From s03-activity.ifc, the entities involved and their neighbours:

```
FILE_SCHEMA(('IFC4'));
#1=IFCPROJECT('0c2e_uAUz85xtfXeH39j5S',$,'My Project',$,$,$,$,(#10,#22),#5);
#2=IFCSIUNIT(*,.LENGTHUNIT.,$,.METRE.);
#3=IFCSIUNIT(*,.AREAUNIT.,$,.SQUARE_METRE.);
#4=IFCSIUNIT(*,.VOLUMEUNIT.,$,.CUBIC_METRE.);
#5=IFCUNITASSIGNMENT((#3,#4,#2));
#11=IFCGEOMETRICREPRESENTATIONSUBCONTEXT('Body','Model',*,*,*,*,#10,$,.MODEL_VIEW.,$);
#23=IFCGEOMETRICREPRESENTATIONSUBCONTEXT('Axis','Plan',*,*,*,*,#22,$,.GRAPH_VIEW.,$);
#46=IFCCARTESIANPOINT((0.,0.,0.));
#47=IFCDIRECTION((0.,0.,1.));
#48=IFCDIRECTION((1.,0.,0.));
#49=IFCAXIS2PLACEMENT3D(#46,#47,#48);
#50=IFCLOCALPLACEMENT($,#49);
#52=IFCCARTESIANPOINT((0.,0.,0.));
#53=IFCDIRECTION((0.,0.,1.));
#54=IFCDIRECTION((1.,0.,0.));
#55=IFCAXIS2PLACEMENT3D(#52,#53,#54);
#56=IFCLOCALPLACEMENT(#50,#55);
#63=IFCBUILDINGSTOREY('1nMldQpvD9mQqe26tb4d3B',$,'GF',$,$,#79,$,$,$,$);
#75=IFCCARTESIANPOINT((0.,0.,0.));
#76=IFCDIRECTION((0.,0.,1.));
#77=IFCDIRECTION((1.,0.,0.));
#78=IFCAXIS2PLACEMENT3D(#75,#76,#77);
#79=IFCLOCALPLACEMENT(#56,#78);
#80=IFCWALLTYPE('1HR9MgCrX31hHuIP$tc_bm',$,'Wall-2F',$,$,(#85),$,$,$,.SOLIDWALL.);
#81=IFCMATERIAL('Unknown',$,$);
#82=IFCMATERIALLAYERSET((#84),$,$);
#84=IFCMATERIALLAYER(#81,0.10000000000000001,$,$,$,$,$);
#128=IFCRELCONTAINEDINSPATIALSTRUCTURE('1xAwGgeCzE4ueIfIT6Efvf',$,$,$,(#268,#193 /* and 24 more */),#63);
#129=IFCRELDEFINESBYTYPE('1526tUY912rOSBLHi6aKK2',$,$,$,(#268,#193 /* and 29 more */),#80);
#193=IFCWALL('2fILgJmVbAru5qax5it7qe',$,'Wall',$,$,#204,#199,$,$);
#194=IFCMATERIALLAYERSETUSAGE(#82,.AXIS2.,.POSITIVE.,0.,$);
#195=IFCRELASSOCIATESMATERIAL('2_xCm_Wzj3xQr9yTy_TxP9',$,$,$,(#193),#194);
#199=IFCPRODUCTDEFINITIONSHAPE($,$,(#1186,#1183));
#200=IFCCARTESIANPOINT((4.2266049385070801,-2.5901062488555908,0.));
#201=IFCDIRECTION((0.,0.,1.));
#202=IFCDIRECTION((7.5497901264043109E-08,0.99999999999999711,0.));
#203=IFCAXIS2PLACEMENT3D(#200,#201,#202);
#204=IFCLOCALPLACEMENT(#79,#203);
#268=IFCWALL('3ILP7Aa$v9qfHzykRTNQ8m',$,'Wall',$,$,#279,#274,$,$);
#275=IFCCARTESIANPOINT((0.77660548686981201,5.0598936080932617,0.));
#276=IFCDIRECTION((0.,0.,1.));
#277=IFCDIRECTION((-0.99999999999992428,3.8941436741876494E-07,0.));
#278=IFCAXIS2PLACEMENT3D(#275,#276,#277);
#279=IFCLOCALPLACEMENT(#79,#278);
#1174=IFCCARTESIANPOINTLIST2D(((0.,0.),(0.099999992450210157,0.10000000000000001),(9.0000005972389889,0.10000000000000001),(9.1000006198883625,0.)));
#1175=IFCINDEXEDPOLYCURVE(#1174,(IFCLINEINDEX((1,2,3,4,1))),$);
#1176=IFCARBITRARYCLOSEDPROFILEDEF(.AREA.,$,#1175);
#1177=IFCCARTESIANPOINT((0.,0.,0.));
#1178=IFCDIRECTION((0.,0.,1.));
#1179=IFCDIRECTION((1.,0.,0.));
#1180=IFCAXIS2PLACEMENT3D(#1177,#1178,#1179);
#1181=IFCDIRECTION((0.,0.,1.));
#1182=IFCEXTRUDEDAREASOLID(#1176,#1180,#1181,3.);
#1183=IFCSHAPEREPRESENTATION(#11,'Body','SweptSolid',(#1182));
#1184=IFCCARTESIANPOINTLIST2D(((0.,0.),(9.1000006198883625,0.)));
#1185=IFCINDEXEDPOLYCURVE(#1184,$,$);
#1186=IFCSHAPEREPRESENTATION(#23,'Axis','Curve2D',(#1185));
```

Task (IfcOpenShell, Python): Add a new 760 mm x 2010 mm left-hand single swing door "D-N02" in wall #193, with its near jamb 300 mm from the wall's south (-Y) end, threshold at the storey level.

```python
import numpy as np
import ifcopenshell
import ifcopenshell.api.feature
import ifcopenshell.api.geometry
import ifcopenshell.api.root
import ifcopenshell.api.spatial
import ifcopenshell.geom
import ifcopenshell.util.element
import ifcopenshell.util.placement
import ifcopenshell.util.representation
import ifcopenshell.util.shape
import ifcopenshell.util.unit

model = ifcopenshell.open("s03-activity.ifc")
unit_scale = ifcopenshell.util.unit.calculate_unit_scale(model)
settings = ifcopenshell.geom.settings()


def volume(element):
    """Net volume in cubic metres, openings subtracted."""
    shape = ifcopenshell.geom.create_shape(settings, element)
    return ifcopenshell.util.shape.get_volume(shape.geometry)


wall = model.by_guid("2fILgJmVbAru5qax5it7qe")
storey = ifcopenshell.util.element.get_container(wall, ifc_class="IfcBuildingStorey")
context = ifcopenshell.util.representation.get_context(model, "Model", "Body", "MODEL_VIEW")
before = volume(wall)

width, height, from_end, sill = 0.76, 2.01, 0.3, 0.0  # metres

# The wall runs along its own X axis, and the end named is its -X end.
wall_shape = ifcopenshell.geom.create_shape(settings, wall)
x, y, z = ifcopenshell.util.shape.get_vertices(wall_shape.geometry).T
start = x.min() + from_end
face, thickness = float(y.min()), float(y.max() - y.min())
wall_matrix = ifcopenshell.util.placement.get_local_placement(wall.ObjectPlacement)
level = ifcopenshell.util.placement.get_local_placement(storey.ObjectPlacement)[2, 3]


def in_wall(x, y):
    """Placement at x, y metres in the wall's axes, at sill height."""
    matrix = wall_matrix.copy()
    matrix[:, 3] = wall_matrix @ np.array([x / unit_scale, y / unit_scale, 0.0, 1.0])
    matrix[2, 3] = level + sill / unit_scale
    return matrix


# Opening: a box that overshoots both wall faces by 50 mm.
opening = ifcopenshell.api.root.create_entity(model, ifc_class="IfcOpeningElement", predefined_type="OPENING")
box = ifcopenshell.api.geometry.add_wall_representation(
    model, context=context, length=width, height=height, thickness=thickness + 0.1
)
ifcopenshell.api.geometry.assign_representation(model, product=opening, representation=box)
ifcopenshell.api.geometry.edit_object_placement(model, product=opening, matrix=in_wall(start, face - 0.05), is_si=False)
ifcopenshell.api.feature.add_feature(model, feature=opening, element=wall)

door = ifcopenshell.api.root.create_entity(model, ifc_class="IfcDoor", name="D-N02", predefined_type="DOOR")
door.OverallWidth, door.OverallHeight = width / unit_scale, height / unit_scale
door.OperationType = "SINGLE_SWING_LEFT"
body = ifcopenshell.api.geometry.add_door_representation(
    model,
    context=context,
    overall_width=door.OverallWidth,
    overall_height=door.OverallHeight,
    operation_type="SINGLE_SWING_LEFT",
    lining_properties={"LiningDepth": thickness / unit_scale, "ThresholdDepth": thickness / unit_scale},
)
ifcopenshell.api.geometry.assign_representation(model, product=door, representation=body)
ifcopenshell.api.spatial.assign_container(model, products=[door], relating_structure=storey)
ifcopenshell.api.feature.add_filling(model, opening=opening, element=door)

# The lining spans the wall, so the door starts at the wall face.
ifcopenshell.api.geometry.edit_object_placement(model, product=door, matrix=in_wall(start, face), is_si=False)

after = volume(wall)

print(f"wall volume {before:.3f} -> {after:.3f} m3")

model.write("s03-activity_v2.ifc")
```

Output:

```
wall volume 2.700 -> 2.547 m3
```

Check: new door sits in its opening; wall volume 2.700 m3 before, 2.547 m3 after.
